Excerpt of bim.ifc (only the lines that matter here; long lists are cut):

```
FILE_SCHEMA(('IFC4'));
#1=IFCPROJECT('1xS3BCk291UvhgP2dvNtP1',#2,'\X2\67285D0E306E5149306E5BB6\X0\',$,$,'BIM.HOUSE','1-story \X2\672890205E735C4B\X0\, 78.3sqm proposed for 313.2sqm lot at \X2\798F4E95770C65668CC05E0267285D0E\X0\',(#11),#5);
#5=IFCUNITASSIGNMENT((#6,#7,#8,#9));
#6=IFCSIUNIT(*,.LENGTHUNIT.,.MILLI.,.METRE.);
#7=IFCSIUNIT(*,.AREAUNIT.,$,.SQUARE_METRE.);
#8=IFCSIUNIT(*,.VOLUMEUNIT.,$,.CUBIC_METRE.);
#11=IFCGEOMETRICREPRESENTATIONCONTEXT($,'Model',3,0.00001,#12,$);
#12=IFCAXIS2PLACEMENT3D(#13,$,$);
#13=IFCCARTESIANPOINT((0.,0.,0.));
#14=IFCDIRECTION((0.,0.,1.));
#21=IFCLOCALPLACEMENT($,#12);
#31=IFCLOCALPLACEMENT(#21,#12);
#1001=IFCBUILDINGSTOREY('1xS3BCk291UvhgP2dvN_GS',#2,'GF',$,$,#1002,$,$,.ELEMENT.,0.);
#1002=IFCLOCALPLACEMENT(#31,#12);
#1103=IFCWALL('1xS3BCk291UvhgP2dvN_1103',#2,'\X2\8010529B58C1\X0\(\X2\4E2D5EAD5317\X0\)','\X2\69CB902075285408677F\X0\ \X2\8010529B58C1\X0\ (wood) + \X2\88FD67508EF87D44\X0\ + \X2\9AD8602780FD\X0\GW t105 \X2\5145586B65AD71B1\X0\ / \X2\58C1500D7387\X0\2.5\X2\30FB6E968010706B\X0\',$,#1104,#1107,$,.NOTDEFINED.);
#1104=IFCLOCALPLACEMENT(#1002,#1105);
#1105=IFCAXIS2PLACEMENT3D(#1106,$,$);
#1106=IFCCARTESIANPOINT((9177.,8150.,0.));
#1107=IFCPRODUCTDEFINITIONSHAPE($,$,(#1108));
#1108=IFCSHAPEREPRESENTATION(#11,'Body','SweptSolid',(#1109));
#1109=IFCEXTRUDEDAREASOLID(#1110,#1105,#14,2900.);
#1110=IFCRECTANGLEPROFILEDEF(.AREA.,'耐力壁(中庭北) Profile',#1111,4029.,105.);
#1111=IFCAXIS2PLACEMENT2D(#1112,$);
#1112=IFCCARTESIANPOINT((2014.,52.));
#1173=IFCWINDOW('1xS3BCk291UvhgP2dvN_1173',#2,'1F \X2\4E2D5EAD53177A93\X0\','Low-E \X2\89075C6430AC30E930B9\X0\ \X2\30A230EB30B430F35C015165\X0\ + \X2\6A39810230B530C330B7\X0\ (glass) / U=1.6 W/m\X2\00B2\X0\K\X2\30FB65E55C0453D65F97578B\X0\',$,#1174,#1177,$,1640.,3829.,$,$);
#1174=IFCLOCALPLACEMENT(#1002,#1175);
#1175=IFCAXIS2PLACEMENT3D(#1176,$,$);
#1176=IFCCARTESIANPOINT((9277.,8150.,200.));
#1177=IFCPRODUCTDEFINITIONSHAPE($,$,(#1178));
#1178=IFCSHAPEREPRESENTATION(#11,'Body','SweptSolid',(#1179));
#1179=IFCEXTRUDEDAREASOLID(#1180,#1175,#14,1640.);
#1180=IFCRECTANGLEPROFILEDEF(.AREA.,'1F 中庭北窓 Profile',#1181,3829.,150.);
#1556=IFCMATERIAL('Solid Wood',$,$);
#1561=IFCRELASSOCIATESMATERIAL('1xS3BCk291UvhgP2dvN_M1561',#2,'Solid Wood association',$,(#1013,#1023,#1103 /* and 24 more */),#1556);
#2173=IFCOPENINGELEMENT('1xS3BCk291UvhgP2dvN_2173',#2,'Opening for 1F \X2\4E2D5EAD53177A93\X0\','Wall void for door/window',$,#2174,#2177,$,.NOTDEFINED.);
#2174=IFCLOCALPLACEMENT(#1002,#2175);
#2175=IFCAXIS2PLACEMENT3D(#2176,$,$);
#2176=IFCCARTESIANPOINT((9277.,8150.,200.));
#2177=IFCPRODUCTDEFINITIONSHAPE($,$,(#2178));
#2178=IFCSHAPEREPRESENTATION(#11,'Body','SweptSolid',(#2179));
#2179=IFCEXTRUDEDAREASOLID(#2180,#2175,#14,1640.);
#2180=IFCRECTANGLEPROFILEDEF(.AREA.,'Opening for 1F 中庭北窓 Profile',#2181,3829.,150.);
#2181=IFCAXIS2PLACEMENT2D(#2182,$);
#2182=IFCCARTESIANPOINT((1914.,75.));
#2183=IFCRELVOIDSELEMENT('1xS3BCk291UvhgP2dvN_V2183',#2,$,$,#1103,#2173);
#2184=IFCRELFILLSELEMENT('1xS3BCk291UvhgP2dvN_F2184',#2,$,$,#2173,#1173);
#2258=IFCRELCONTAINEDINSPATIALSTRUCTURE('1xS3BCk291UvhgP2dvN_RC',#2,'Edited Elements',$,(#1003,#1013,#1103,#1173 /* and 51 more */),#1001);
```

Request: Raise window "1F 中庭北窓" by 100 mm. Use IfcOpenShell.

```python
import numpy as np
import ifcopenshell
import ifcopenshell.api.geometry
import ifcopenshell.util.placement
import ifcopenshell.util.unit

model = ifcopenshell.open("bim.ifc")
unit_scale = ifcopenshell.util.unit.calculate_unit_scale(model)

window = model.by_guid("1xS3BCk291UvhgP2dvN_1173")
opening = window.FillsVoids[0].RelatingOpeningElement
dz = 100.0

shift = np.array([0.0, 0.0, dz])
# The window is not placed relative to its opening, so move both.
for product in (opening, window):
    matrix = ifcopenshell.util.placement.get_local_placement(product.ObjectPlacement)
    matrix[:3, 3] += shift
    ifcopenshell.api.geometry.edit_object_placement(model, product=product, matrix=matrix, is_si=False)

print(f"moved by {dz * unit_scale:+.3f} m")

model.write("bim_rev.ifc")
```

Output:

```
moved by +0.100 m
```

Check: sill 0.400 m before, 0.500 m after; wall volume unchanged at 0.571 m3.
